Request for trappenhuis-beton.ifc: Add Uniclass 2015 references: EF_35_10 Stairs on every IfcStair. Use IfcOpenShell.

First a look at what the model holds.

```python
import ifcopenshell

model = ifcopenshell.open("trappenhuis-beton.ifc")
print(model.schema)
print("classifications:", [c.Name for c in model.by_type("IfcClassification")])
for ifc_class in ("IfcDoor", "IfcRoof", "IfcStair", "IfcWall", "IfcWindow"):
    print(ifc_class, len(model.by_type(ifc_class)))
```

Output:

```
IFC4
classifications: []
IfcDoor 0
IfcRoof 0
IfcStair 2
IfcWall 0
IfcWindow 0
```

```python
import ifcopenshell
import ifcopenshell.api.classification

model = ifcopenshell.open("trappenhuis-beton.ifc")

system = ifcopenshell.api.classification.add_classification(model, classification="Uniclass 2015")

codes = {
    "IfcStair": ("EF_35_10", "Stairs"),
}
for ifc_class, (code, name) in codes.items():
    products = model.by_type(ifc_class)
    ifcopenshell.api.classification.add_reference(
        model, products=products, classification=system, identification=code, name=name
    )
    print(code, len(products))

model.write("trappenhuis-beton_edited.ifc")
```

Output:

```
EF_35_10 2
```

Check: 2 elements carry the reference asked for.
